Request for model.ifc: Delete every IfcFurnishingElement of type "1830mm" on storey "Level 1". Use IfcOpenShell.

First a look at what the model holds.

```python
import ifcopenshell
import ifcopenshell.util.element

model = ifcopenshell.open("model.ifc")
print(model.schema)
storey = next(s for s in model.by_type("IfcBuildingStorey") if s.Name == "Level 1")
furniture = [e for e in ifcopenshell.util.element.get_decomposition(storey) if e.is_a("IfcFurnishingElement")]
seen = {}
for e in furniture:
    element_type = ifcopenshell.util.element.get_type(e)
    name = element_type.Name if element_type not in (None, e) else None
    seen[name] = seen.get(name, 0) + 1
for name, count in sorted(seen.items(), key=str):
    print(count, "x", name)
```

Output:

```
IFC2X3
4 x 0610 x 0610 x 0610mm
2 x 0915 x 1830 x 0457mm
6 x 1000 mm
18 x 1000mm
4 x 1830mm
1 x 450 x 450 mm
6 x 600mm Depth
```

```python
import ifcopenshell
import ifcopenshell.api.root
import ifcopenshell.util.element

model = ifcopenshell.open("model.ifc")

storey = next(s for s in model.by_type("IfcBuildingStorey") if s.Name == "Level 1")
furniture = [e for e in ifcopenshell.util.element.get_decomposition(storey) if e.is_a("IfcFurnishingElement")]
targets = [e for e in furniture if (t := ifcopenshell.util.element.get_type(e)) not in (None, e) and t.Name == "1830mm"]

for e in targets:
    ifcopenshell.api.root.remove_product(model, product=e)
print(len(targets), "removed")

model.write("model_updated.ifc")
```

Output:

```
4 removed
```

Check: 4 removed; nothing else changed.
